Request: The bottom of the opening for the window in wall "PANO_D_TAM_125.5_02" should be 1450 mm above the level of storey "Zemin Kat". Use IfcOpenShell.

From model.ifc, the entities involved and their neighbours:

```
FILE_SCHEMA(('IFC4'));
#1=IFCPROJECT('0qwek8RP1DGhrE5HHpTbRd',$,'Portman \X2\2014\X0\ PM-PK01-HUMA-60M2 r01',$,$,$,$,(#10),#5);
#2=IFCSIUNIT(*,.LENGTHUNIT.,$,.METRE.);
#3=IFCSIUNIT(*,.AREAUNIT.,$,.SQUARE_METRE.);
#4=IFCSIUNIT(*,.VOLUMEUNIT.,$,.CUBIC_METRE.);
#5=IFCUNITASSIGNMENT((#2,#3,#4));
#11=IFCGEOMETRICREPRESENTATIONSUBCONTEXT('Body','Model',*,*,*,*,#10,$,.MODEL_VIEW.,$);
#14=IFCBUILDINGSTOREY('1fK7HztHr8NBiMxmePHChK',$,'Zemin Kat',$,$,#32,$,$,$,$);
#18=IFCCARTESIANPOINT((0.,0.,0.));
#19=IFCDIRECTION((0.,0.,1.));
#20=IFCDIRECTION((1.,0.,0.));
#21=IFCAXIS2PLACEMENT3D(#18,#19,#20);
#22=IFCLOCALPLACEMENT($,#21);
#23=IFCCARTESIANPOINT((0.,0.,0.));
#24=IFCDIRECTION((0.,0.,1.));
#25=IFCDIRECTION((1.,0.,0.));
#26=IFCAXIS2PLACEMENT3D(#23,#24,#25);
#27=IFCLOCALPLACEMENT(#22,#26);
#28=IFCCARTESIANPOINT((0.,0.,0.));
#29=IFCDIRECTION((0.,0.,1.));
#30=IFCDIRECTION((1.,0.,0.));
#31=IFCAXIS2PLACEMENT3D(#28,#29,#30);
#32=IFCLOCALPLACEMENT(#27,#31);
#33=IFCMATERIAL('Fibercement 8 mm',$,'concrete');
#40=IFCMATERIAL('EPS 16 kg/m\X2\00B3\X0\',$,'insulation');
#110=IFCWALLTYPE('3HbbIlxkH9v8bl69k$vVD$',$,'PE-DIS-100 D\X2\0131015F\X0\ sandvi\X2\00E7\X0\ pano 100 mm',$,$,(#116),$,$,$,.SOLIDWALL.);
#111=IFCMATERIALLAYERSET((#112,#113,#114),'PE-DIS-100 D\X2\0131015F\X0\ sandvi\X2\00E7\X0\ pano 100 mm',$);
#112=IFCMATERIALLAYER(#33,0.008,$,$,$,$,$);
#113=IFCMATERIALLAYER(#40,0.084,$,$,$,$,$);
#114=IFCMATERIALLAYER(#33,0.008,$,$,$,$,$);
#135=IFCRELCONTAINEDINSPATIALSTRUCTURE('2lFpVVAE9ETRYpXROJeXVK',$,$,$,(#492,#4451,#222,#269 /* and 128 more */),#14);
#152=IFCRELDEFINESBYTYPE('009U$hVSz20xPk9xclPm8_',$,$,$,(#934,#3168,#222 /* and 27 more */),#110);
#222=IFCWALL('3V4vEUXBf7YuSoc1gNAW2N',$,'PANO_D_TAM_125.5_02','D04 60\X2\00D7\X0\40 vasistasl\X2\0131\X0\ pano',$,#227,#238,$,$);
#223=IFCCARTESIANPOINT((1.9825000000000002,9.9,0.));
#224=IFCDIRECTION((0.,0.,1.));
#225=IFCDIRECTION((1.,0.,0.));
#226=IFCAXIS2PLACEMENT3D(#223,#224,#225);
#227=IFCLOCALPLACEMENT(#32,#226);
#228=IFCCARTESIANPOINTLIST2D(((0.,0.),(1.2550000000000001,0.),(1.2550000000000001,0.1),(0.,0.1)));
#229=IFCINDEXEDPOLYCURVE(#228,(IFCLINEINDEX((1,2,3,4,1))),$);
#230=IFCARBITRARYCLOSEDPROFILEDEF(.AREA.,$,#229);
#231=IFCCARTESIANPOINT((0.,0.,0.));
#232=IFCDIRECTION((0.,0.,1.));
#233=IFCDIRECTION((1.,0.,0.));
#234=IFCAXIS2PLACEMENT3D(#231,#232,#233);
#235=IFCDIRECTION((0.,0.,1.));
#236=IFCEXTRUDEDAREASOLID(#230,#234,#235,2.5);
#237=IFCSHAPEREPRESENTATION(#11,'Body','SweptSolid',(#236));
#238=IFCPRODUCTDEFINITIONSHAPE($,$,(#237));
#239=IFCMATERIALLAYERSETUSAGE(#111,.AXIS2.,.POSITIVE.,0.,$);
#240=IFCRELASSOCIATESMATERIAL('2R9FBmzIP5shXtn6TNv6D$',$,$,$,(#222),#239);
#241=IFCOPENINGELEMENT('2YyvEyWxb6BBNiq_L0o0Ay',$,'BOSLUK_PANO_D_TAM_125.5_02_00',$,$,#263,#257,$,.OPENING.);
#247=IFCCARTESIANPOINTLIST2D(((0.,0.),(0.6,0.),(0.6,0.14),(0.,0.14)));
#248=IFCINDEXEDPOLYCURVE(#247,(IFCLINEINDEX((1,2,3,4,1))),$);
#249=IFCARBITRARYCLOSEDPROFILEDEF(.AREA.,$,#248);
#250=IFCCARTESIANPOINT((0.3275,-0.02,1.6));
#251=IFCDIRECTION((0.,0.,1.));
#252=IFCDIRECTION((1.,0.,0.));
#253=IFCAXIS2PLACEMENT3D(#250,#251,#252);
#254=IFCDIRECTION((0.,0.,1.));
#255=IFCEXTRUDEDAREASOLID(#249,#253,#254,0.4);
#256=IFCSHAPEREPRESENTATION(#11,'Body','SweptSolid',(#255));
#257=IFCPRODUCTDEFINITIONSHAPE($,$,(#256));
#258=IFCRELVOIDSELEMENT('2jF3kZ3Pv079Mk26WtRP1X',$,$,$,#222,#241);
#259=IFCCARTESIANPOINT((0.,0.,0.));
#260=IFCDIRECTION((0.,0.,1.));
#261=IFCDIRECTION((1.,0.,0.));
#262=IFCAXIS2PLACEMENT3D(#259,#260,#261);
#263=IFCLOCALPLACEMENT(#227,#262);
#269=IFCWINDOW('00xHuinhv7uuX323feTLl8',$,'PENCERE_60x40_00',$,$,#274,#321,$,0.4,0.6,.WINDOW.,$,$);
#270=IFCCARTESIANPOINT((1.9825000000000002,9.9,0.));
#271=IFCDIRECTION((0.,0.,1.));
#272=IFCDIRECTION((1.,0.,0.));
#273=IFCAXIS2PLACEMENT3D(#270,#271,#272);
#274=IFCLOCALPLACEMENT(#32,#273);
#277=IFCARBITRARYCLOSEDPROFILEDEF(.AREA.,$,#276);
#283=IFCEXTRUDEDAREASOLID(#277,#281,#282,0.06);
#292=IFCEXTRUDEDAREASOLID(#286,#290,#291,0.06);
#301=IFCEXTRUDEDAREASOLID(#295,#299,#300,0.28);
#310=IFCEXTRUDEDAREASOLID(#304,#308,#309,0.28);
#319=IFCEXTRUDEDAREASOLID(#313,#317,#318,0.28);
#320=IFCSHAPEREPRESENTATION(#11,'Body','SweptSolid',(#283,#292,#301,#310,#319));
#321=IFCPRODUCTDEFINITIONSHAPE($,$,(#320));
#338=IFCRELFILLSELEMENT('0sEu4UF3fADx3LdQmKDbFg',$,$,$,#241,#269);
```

```python
import numpy as np
import ifcopenshell
import ifcopenshell.api.geometry
import ifcopenshell.geom
import ifcopenshell.util.element
import ifcopenshell.util.placement
import ifcopenshell.util.shape
import ifcopenshell.util.unit

model = ifcopenshell.open("model.ifc")
unit_scale = ifcopenshell.util.unit.calculate_unit_scale(model)

window = model.by_guid("00xHuinhv7uuX323feTLl8")
opening = window.FillsVoids[0].RelatingOpeningElement
storey = ifcopenshell.util.element.get_container(window, ifc_class="IfcBuildingStorey")
level = ifcopenshell.util.placement.get_local_placement(storey.ObjectPlacement)[2, 3]

# The opening's origin need not be at the sill, so measure its lowest point.
shape = ifcopenshell.geom.create_shape(ifcopenshell.geom.settings(), opening)
bottom = ifcopenshell.util.shape.get_shape_bottom_elevation(shape, shape.geometry) / unit_scale
dz = level + 1.45 / unit_scale - bottom

shift = np.array([0.0, 0.0, dz])
# The window is not placed relative to its opening, so move both.
for product in (opening, window):
    matrix = ifcopenshell.util.placement.get_local_placement(product.ObjectPlacement)
    matrix[:3, 3] += shift
    ifcopenshell.api.geometry.edit_object_placement(model, product=product, matrix=matrix, is_si=False)

print(f"moved by {dz * unit_scale:+.3f} m")

model.write("model_updated.ifc")
```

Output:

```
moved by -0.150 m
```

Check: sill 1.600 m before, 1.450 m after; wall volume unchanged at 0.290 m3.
